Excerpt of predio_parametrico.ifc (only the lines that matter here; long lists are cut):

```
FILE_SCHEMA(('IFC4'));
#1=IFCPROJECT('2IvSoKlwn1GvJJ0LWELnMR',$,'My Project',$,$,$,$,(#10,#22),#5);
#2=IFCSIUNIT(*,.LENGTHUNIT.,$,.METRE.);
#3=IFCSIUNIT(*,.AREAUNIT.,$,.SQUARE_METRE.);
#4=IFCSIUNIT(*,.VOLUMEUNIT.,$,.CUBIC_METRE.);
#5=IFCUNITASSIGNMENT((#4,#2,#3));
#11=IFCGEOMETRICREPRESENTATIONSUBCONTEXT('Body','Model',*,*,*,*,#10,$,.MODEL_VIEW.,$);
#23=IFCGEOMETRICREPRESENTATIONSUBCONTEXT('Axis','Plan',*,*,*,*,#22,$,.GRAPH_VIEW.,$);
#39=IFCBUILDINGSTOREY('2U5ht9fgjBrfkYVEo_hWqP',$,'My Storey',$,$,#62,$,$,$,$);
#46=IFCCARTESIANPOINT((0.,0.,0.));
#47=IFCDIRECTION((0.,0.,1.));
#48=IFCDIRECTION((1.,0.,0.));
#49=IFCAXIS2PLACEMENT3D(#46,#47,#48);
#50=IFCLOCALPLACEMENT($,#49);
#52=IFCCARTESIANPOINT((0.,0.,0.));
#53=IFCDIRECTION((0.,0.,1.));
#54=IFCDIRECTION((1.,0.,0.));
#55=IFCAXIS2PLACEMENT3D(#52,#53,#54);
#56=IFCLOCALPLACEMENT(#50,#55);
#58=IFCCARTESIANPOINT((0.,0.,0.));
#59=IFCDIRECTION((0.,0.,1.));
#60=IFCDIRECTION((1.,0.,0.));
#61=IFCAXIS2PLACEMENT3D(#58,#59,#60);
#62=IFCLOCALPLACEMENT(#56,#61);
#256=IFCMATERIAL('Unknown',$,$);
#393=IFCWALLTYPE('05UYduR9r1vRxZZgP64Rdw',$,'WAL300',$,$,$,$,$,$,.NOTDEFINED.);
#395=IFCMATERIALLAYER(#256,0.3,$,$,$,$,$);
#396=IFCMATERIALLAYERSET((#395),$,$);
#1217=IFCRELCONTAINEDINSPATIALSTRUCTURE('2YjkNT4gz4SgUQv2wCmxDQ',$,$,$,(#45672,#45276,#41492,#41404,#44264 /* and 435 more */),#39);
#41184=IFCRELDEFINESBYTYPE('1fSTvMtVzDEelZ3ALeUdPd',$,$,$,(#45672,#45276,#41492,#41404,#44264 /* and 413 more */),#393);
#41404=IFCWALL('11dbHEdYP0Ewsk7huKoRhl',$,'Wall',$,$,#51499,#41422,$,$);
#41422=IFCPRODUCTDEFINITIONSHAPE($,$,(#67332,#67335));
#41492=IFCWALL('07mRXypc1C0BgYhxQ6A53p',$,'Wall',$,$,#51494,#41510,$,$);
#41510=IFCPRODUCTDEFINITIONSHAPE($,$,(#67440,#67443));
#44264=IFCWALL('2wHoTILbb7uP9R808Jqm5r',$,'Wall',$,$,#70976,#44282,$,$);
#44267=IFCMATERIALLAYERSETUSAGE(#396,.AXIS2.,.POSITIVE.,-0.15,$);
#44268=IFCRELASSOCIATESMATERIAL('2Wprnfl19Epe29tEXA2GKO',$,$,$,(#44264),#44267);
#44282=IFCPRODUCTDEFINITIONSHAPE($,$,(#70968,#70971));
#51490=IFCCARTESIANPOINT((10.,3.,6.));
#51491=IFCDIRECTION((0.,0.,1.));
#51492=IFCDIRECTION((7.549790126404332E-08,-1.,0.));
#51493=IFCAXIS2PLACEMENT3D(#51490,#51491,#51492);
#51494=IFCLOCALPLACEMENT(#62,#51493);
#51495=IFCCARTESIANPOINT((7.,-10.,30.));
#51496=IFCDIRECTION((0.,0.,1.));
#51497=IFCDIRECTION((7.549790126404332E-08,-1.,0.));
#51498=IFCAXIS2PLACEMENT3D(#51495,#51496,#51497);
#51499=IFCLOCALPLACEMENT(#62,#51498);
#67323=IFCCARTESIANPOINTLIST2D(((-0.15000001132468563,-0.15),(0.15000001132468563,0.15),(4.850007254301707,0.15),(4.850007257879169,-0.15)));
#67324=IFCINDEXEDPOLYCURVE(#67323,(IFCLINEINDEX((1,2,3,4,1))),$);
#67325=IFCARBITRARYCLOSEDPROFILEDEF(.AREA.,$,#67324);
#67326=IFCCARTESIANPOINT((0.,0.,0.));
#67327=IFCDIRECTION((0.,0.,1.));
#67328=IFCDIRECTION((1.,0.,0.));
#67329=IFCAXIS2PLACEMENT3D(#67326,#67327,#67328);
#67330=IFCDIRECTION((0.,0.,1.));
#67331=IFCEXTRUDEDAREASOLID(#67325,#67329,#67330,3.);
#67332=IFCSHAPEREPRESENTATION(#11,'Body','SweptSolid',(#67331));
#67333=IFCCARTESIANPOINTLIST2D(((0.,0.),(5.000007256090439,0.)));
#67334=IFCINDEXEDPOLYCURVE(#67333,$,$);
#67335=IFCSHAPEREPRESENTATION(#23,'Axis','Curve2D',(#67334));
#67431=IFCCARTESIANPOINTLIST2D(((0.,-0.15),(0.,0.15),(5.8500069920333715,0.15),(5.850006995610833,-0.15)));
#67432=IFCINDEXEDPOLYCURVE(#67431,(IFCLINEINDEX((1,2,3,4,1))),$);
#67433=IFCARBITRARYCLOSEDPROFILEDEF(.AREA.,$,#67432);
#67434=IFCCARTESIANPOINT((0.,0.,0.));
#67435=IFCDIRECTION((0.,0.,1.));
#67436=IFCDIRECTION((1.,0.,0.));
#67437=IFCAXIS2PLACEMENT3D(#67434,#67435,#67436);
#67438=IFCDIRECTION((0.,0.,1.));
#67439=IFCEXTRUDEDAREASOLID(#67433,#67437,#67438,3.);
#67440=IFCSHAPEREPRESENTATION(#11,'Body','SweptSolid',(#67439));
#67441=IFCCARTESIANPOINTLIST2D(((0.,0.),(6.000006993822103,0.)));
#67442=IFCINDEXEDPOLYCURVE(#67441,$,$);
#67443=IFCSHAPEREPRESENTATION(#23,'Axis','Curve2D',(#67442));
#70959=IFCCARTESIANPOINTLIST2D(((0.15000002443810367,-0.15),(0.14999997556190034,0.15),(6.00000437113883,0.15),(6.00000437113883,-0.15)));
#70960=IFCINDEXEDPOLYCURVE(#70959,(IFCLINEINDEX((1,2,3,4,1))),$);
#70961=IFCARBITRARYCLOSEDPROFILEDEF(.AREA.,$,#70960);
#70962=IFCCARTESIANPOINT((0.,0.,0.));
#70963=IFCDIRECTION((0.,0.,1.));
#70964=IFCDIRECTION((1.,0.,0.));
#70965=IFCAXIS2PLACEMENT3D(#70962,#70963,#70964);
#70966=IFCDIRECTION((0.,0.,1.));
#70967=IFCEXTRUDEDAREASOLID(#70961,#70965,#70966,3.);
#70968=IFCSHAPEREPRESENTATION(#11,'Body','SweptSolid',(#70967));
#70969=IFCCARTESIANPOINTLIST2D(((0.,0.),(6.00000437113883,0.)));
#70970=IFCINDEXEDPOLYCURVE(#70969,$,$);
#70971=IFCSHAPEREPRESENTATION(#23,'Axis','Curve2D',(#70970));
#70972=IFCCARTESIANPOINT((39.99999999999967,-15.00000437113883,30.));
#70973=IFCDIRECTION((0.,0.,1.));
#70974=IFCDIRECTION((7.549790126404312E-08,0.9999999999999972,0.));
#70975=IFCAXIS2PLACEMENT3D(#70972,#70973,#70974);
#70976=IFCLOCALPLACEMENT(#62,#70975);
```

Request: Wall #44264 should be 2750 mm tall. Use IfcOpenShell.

```python
import ifcopenshell
import ifcopenshell.geom
import ifcopenshell.util.representation
import ifcopenshell.util.shape
import ifcopenshell.util.unit

model = ifcopenshell.open("predio_parametrico.ifc")
unit_scale = ifcopenshell.util.unit.calculate_unit_scale(model)
settings = ifcopenshell.geom.settings()


def volume(element):
    """Net volume in cubic metres, openings subtracted."""
    shape = ifcopenshell.geom.create_shape(settings, element)
    return ifcopenshell.util.shape.get_volume(shape.geometry)


wall = model.by_id(44264)
before = volume(wall)

body = ifcopenshell.util.representation.get_representation(wall, "Model", "Body")
solid = body.Items[0]
old_height = solid.Depth
solid.Depth = 2.75 / unit_scale
after = volume(wall)

print(f"height {old_height:g} -> {solid.Depth:g}, volume {before:.3f} -> {after:.3f} m3")

model.write("predio_parametrico-out.ifc")
```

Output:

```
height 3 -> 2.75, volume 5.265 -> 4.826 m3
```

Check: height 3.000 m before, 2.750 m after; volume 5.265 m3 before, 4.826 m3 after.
